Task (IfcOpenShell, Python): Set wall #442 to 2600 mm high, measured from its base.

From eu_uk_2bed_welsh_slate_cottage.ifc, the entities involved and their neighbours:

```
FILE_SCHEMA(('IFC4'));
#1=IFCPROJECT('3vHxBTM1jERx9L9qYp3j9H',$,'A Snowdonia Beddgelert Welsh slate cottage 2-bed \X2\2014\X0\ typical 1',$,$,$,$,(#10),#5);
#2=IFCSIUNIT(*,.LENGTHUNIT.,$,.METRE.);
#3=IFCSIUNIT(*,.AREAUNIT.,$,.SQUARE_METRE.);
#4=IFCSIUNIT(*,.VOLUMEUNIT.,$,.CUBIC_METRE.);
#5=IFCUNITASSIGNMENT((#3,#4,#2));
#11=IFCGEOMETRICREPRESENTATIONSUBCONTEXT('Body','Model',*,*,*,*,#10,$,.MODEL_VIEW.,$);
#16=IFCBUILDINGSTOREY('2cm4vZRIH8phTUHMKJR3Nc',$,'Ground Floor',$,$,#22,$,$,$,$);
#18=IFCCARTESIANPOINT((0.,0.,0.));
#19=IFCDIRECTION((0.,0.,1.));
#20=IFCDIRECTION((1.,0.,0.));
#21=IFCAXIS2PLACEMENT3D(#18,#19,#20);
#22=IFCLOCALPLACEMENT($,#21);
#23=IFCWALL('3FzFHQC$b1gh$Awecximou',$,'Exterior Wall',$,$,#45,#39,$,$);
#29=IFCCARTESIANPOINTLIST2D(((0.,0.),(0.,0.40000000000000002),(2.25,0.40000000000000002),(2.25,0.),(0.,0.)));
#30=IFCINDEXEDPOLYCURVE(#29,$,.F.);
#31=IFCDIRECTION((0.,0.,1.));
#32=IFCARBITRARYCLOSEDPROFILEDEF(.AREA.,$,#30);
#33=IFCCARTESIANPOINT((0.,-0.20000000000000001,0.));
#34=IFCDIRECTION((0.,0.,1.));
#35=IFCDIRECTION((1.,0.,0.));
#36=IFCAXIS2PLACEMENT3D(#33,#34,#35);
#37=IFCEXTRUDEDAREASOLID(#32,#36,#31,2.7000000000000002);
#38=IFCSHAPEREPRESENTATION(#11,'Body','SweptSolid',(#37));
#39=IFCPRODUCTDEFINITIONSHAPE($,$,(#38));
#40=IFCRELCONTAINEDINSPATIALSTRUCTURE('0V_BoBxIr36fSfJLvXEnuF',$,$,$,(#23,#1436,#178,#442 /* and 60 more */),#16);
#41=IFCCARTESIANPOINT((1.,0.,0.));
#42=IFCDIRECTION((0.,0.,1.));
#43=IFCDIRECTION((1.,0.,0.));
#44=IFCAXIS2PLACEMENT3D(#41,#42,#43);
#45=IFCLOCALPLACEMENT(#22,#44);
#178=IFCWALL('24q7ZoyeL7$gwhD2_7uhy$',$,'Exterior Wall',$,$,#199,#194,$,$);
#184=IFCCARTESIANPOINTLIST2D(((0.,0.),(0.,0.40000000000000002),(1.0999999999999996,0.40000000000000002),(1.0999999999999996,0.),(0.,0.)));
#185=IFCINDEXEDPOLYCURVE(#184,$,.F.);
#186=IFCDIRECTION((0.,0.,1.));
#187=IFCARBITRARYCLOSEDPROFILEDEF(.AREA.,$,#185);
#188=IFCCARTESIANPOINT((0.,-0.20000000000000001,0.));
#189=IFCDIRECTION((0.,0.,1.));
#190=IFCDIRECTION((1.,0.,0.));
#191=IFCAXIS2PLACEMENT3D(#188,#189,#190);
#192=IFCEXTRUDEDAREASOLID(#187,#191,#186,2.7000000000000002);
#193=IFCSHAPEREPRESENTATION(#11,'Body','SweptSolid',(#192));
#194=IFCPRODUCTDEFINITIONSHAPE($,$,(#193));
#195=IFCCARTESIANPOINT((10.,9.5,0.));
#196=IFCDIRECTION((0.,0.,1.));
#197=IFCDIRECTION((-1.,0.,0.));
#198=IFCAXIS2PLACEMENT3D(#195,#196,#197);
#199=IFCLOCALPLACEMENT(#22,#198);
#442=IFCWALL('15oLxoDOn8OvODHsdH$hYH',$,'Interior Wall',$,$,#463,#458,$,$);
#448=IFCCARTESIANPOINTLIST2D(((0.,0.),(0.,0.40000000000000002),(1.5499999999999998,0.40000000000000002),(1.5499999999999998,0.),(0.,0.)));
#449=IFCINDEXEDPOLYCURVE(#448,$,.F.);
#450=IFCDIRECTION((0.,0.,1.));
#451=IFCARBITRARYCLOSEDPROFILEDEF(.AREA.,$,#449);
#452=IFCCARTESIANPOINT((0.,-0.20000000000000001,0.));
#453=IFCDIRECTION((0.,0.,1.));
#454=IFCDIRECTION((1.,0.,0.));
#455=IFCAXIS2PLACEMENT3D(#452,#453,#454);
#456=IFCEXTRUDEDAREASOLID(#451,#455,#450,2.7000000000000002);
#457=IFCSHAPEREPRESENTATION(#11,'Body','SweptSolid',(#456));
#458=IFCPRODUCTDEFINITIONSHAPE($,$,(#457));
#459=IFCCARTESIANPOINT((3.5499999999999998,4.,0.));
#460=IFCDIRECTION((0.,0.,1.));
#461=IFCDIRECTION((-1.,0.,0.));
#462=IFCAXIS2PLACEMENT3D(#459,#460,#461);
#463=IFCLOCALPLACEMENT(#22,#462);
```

```python
import ifcopenshell
import ifcopenshell.geom
import ifcopenshell.util.representation
import ifcopenshell.util.shape
import ifcopenshell.util.unit

model = ifcopenshell.open("eu_uk_2bed_welsh_slate_cottage.ifc")
unit_scale = ifcopenshell.util.unit.calculate_unit_scale(model)
settings = ifcopenshell.geom.settings()


def volume(element):
    """Net volume in cubic metres, openings subtracted."""
    shape = ifcopenshell.geom.create_shape(settings, element)
    return ifcopenshell.util.shape.get_volume(shape.geometry)


wall = model.by_guid("15oLxoDOn8OvODHsdH$hYH")
before = volume(wall)

body = ifcopenshell.util.representation.get_representation(wall, "Model", "Body")
solid = body.Items[0]
old_height = solid.Depth
solid.Depth = 2.6 / unit_scale
after = volume(wall)

print(f"height {old_height:g} -> {solid.Depth:g}, volume {before:.3f} -> {after:.3f} m3")

model.write("eu_uk_2bed_welsh_slate_cottage_rev.ifc")
```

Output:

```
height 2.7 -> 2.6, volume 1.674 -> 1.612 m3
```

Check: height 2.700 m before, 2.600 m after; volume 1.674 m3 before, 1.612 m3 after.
